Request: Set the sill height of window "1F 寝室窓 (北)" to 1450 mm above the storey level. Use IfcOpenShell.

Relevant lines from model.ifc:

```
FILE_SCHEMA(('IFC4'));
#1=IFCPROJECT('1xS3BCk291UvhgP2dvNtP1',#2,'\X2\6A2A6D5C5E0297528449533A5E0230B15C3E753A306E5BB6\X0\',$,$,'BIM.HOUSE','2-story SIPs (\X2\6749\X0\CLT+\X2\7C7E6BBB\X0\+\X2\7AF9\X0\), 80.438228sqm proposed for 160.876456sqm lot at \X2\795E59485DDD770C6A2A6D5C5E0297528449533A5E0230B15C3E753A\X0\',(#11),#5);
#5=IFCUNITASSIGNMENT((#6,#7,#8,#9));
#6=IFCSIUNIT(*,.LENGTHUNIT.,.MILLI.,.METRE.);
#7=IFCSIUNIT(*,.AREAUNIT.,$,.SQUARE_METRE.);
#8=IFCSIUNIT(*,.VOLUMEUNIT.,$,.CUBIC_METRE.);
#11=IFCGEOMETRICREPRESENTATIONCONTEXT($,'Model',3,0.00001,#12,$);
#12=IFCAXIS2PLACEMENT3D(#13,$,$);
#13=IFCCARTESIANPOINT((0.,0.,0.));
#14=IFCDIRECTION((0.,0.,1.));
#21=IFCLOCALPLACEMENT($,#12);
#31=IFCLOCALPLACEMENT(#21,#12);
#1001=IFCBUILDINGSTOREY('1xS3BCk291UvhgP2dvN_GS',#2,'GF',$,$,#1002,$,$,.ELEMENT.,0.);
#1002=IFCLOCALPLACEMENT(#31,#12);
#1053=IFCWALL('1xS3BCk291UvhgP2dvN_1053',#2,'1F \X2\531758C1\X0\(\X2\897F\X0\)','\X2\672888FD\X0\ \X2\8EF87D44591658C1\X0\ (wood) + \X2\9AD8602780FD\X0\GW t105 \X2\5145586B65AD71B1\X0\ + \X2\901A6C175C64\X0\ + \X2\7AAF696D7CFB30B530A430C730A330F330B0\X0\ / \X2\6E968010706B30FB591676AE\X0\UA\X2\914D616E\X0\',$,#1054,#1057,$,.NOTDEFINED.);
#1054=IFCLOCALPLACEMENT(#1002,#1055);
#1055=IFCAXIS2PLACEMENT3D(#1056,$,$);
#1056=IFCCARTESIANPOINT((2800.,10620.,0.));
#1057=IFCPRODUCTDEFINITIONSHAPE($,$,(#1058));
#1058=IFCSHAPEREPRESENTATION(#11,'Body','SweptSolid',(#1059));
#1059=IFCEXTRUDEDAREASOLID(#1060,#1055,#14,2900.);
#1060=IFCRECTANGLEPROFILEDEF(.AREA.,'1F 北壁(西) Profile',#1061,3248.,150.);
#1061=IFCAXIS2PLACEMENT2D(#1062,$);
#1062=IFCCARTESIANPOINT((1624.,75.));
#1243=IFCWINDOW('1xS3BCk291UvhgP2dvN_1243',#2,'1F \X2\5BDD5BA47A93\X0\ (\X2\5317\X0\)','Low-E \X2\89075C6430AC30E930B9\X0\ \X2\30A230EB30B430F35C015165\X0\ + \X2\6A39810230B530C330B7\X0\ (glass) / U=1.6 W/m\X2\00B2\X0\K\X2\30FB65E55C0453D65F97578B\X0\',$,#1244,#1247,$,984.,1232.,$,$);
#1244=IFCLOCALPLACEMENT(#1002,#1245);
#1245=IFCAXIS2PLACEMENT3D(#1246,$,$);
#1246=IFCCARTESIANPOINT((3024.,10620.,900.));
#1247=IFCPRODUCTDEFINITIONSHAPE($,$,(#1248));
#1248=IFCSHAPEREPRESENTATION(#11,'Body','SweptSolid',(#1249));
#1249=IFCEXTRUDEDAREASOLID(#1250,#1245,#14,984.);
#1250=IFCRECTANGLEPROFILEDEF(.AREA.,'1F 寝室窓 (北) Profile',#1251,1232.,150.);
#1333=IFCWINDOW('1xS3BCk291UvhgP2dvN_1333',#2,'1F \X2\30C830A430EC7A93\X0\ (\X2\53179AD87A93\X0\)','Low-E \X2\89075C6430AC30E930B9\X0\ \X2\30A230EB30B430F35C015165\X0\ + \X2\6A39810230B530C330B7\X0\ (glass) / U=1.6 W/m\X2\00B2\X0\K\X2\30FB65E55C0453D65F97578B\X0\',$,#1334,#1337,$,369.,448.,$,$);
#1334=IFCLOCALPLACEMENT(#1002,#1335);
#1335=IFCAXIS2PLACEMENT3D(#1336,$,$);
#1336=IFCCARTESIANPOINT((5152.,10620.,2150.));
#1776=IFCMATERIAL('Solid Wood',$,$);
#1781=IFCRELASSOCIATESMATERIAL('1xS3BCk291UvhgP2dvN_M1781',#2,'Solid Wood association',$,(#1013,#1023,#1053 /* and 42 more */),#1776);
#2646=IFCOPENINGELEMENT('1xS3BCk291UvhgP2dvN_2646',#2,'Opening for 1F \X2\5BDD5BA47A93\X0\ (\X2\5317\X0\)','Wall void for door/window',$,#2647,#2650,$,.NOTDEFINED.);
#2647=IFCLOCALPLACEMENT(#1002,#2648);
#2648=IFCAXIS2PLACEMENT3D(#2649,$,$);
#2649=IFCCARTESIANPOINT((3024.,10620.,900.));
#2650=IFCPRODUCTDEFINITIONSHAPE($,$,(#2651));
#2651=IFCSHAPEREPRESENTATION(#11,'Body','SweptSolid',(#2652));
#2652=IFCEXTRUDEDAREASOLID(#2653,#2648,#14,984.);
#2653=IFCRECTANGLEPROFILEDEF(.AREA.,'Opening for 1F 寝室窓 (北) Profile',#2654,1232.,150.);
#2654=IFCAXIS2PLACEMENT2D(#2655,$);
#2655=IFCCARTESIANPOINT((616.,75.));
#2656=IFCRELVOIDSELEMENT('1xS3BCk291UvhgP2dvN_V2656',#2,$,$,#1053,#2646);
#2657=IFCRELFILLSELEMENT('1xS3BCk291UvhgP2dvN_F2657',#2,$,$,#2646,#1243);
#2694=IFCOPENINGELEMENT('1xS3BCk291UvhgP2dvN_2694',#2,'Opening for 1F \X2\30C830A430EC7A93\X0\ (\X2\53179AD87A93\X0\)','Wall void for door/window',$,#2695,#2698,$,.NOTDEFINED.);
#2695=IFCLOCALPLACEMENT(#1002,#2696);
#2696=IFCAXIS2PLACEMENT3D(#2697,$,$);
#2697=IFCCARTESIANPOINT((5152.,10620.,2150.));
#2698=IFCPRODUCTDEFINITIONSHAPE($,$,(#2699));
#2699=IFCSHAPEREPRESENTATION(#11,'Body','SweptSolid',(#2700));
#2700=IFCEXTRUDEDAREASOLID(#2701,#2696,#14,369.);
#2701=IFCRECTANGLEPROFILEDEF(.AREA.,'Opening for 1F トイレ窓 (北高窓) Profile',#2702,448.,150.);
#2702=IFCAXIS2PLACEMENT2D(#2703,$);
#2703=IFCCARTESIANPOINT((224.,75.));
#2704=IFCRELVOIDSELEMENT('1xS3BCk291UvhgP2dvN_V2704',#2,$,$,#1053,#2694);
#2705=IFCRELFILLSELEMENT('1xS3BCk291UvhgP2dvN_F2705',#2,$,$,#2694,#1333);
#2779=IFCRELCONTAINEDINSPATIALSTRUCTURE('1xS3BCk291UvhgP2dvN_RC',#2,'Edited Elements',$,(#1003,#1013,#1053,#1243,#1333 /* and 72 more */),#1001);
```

```python
import numpy as np
import ifcopenshell
import ifcopenshell.api.geometry
import ifcopenshell.geom
import ifcopenshell.util.element
import ifcopenshell.util.placement
import ifcopenshell.util.shape
import ifcopenshell.util.unit

model = ifcopenshell.open("model.ifc")
unit_scale = ifcopenshell.util.unit.calculate_unit_scale(model)

window = model.by_guid("1xS3BCk291UvhgP2dvN_1243")
opening = window.FillsVoids[0].RelatingOpeningElement
storey = ifcopenshell.util.element.get_container(window, ifc_class="IfcBuildingStorey")
level = ifcopenshell.util.placement.get_local_placement(storey.ObjectPlacement)[2, 3]

# The opening's origin need not be at the sill, so measure its lowest point.
shape = ifcopenshell.geom.create_shape(ifcopenshell.geom.settings(), opening)
bottom = ifcopenshell.util.shape.get_shape_bottom_elevation(shape, shape.geometry) / unit_scale
dz = level + 1450.0 - bottom

shift = np.array([0.0, 0.0, dz])
# The window is not placed relative to its opening, so move both.
for product in (opening, window):
    matrix = ifcopenshell.util.placement.get_local_placement(product.ObjectPlacement)
    matrix[:3, 3] += shift
    ifcopenshell.api.geometry.edit_object_placement(model, product=product, matrix=matrix, is_si=False)

print(f"moved by {dz * unit_scale:+.3f} m")

model.write("model_rev.ifc")
```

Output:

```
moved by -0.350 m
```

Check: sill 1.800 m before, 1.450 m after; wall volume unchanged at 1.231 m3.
